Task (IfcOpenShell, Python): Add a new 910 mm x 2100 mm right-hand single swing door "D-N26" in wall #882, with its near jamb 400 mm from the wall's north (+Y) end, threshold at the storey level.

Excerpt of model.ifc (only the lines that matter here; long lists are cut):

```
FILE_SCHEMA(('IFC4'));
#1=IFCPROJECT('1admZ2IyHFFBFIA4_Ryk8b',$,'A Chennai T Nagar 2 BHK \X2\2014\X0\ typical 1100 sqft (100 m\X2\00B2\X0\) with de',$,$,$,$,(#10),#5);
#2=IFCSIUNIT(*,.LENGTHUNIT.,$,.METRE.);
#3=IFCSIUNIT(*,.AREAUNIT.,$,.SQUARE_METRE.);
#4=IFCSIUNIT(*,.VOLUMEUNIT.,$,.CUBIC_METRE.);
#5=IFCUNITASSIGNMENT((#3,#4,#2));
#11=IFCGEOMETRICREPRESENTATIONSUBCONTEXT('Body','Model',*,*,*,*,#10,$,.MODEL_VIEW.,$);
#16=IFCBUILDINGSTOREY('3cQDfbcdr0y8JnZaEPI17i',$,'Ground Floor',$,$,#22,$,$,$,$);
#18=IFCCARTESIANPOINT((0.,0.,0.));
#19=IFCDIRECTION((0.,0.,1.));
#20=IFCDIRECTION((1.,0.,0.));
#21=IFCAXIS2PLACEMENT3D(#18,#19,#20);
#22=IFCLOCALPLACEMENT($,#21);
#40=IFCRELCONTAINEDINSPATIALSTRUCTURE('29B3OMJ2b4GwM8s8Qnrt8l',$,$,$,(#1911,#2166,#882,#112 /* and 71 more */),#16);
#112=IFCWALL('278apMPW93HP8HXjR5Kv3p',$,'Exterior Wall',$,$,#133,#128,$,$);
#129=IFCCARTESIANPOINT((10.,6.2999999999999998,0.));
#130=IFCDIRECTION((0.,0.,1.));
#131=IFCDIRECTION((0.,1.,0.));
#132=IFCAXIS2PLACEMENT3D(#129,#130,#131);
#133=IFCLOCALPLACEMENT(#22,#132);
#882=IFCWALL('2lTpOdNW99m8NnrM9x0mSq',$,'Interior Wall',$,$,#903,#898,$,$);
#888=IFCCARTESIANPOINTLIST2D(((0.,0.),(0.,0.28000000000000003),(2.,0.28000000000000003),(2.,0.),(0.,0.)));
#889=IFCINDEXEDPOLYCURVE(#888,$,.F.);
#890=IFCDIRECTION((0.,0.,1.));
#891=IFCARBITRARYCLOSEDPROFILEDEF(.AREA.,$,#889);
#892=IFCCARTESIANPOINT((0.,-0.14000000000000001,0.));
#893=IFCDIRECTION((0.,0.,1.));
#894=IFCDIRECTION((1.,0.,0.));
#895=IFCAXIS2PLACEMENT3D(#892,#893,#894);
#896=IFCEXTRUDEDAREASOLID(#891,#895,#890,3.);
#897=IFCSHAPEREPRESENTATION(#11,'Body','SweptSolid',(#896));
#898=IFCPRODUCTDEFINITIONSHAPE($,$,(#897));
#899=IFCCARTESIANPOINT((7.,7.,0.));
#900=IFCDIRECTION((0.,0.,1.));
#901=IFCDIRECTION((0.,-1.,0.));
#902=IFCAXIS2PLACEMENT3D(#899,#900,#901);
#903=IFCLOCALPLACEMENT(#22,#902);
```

```python
import numpy as np
import ifcopenshell
import ifcopenshell.api.feature
import ifcopenshell.api.geometry
import ifcopenshell.api.root
import ifcopenshell.api.spatial
import ifcopenshell.geom
import ifcopenshell.util.element
import ifcopenshell.util.placement
import ifcopenshell.util.representation
import ifcopenshell.util.shape
import ifcopenshell.util.unit

model = ifcopenshell.open("model.ifc")
unit_scale = ifcopenshell.util.unit.calculate_unit_scale(model)
settings = ifcopenshell.geom.settings()


def volume(element):
    """Net volume in cubic metres, openings subtracted."""
    shape = ifcopenshell.geom.create_shape(settings, element)
    return ifcopenshell.util.shape.get_volume(shape.geometry)


wall = model.by_id(882)
storey = ifcopenshell.util.element.get_container(wall, ifc_class="IfcBuildingStorey")
context = ifcopenshell.util.representation.get_context(model, "Model", "Body", "MODEL_VIEW")
before = volume(wall)

width, height, from_end, sill = 0.91, 2.1, 0.4, 0.0  # metres

# The wall runs along its own X axis, and the end named is its -X end.
wall_shape = ifcopenshell.geom.create_shape(settings, wall)
x, y, z = ifcopenshell.util.shape.get_vertices(wall_shape.geometry).T
start = x.min() + from_end
face, thickness = float(y.min()), float(y.max() - y.min())
wall_matrix = ifcopenshell.util.placement.get_local_placement(wall.ObjectPlacement)
level = ifcopenshell.util.placement.get_local_placement(storey.ObjectPlacement)[2, 3]


def in_wall(x, y):
    """Placement at x, y metres in the wall's axes, at sill height."""
    matrix = wall_matrix.copy()
    matrix[:, 3] = wall_matrix @ np.array([x / unit_scale, y / unit_scale, 0.0, 1.0])
    matrix[2, 3] = level + sill / unit_scale
    return matrix


# Opening: a box that overshoots both wall faces by 50 mm.
opening = ifcopenshell.api.root.create_entity(model, ifc_class="IfcOpeningElement", predefined_type="OPENING")
box = ifcopenshell.api.geometry.add_wall_representation(
    model, context=context, length=width, height=height, thickness=thickness + 0.1
)
ifcopenshell.api.geometry.assign_representation(model, product=opening, representation=box)
ifcopenshell.api.geometry.edit_object_placement(model, product=opening, matrix=in_wall(start, face - 0.05), is_si=False)
ifcopenshell.api.feature.add_feature(model, feature=opening, element=wall)

door = ifcopenshell.api.root.create_entity(model, ifc_class="IfcDoor", name="D-N26", predefined_type="DOOR")
door.OverallWidth, door.OverallHeight = width / unit_scale, height / unit_scale
door.OperationType = "SINGLE_SWING_RIGHT"
body = ifcopenshell.api.geometry.add_door_representation(
    model,
    context=context,
    overall_width=door.OverallWidth,
    overall_height=door.OverallHeight,
    operation_type="SINGLE_SWING_RIGHT",
    lining_properties={"LiningDepth": thickness / unit_scale, "ThresholdDepth": thickness / unit_scale},
)
ifcopenshell.api.geometry.assign_representation(model, product=door, representation=body)
ifcopenshell.api.spatial.assign_container(model, products=[door], relating_structure=storey)
ifcopenshell.api.feature.add_filling(model, opening=opening, element=door)

# The lining spans the wall, so the door starts at the wall face.
ifcopenshell.api.geometry.edit_object_placement(model, product=door, matrix=in_wall(start, face), is_si=False)

after = volume(wall)

print(f"wall volume {before:.3f} -> {after:.3f} m3")

model.write("model_v2.ifc")
```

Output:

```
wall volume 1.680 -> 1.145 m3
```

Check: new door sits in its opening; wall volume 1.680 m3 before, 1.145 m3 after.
